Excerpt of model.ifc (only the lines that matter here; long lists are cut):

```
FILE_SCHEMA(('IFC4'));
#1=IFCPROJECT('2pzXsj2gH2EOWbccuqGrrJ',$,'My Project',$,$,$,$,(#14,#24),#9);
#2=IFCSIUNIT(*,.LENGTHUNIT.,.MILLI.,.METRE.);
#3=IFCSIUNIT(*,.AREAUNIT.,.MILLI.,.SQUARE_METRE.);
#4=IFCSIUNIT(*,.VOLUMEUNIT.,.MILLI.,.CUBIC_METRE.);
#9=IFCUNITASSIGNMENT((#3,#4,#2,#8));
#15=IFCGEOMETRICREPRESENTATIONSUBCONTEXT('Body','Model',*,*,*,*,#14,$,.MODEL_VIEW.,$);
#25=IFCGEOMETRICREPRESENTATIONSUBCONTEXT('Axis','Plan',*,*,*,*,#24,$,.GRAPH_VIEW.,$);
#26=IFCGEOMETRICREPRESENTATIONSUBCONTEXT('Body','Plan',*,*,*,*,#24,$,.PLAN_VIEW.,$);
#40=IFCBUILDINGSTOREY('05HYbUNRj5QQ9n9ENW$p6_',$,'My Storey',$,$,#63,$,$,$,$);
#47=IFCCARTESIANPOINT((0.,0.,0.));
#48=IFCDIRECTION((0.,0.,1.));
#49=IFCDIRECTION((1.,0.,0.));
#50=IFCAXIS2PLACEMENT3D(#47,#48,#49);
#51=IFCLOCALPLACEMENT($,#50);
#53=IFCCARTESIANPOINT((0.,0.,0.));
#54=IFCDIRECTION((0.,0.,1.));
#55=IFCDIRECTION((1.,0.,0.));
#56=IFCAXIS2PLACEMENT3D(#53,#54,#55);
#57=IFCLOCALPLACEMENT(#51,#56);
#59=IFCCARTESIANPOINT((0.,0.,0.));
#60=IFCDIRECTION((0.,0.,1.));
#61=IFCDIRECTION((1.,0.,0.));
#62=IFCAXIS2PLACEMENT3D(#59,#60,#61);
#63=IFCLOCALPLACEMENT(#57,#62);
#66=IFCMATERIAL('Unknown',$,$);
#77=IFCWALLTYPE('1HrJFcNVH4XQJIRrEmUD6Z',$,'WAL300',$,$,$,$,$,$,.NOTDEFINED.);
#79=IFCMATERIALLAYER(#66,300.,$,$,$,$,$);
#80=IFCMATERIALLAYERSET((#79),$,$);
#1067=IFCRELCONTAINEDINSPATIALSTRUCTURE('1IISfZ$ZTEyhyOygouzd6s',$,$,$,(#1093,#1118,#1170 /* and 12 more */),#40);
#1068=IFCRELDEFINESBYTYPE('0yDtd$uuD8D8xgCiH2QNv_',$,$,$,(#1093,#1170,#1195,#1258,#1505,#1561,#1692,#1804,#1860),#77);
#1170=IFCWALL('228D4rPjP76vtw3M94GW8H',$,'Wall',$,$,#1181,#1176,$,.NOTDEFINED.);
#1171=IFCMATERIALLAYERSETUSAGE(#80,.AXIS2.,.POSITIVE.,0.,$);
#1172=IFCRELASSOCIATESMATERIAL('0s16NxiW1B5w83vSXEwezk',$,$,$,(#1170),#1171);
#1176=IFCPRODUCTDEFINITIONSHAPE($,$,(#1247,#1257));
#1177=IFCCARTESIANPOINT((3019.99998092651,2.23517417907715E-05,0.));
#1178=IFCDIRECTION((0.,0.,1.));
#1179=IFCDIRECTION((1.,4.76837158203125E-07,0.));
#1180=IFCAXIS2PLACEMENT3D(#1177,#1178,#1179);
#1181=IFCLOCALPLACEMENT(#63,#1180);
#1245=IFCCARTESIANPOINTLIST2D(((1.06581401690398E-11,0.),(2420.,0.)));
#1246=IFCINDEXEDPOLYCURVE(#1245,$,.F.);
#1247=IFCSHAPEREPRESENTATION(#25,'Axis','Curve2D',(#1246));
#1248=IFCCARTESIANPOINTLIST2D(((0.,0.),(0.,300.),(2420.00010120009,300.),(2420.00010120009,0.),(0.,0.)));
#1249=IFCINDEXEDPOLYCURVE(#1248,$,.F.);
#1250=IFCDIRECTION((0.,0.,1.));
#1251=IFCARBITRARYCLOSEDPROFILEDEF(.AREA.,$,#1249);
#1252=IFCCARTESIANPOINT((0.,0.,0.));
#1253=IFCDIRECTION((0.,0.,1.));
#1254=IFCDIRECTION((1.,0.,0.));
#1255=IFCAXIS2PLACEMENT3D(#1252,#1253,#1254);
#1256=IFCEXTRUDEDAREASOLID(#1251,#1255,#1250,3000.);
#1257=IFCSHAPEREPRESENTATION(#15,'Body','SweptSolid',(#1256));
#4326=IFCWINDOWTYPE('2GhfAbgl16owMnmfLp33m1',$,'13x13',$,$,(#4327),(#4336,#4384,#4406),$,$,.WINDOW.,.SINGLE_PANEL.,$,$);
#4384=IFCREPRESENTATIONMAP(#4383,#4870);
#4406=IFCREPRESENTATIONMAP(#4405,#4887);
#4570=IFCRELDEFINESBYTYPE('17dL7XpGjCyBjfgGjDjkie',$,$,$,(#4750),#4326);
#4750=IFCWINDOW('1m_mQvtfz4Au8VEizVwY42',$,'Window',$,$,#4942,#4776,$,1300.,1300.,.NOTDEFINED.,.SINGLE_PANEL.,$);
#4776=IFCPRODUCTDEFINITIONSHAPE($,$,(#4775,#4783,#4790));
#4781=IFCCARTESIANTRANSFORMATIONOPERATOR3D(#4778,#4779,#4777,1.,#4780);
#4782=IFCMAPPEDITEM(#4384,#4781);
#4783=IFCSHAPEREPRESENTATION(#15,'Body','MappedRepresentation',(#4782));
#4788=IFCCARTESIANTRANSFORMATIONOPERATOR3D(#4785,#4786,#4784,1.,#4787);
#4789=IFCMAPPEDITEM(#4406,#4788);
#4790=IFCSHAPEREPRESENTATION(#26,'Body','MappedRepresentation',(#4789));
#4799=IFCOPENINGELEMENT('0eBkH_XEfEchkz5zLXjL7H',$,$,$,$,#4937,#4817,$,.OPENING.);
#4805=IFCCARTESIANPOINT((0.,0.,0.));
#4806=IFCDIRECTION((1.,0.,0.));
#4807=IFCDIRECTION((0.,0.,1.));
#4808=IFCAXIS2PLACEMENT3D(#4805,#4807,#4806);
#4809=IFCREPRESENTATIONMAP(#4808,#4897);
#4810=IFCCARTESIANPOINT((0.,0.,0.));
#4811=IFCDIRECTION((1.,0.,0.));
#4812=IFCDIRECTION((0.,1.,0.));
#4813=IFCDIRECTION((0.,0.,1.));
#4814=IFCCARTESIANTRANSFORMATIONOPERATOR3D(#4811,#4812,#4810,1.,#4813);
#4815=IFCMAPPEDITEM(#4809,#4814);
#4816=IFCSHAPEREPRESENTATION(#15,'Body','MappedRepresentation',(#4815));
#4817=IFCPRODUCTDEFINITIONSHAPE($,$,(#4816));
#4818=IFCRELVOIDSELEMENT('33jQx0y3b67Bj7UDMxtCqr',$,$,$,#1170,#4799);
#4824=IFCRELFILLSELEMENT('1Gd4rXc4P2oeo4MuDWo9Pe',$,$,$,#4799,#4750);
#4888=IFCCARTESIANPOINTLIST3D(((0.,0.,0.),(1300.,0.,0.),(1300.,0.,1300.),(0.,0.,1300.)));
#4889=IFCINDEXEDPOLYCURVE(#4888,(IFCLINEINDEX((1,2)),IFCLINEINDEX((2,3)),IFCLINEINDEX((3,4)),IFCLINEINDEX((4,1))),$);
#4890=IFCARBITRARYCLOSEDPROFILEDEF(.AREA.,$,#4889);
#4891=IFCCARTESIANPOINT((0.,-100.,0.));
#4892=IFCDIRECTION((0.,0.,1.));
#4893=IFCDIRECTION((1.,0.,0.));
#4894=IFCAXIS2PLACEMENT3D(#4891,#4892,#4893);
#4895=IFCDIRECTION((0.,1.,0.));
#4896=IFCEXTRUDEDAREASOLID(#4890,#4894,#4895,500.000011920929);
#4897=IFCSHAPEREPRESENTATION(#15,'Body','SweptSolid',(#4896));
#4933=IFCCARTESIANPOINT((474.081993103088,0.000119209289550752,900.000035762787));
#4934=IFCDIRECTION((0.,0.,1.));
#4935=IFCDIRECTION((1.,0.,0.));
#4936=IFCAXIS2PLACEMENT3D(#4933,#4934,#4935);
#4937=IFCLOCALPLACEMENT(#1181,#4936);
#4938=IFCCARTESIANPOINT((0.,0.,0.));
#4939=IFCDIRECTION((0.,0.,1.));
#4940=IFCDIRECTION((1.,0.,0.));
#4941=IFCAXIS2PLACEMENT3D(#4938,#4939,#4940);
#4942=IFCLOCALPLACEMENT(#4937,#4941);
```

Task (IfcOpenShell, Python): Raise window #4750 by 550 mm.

```python
import numpy as np
import ifcopenshell
import ifcopenshell.api.geometry
import ifcopenshell.util.placement
import ifcopenshell.util.unit

model = ifcopenshell.open("model.ifc")
unit_scale = ifcopenshell.util.unit.calculate_unit_scale(model)

window = model.by_guid("1m_mQvtfz4Au8VEizVwY42")
opening = window.FillsVoids[0].RelatingOpeningElement
dz = 0.55 / unit_scale

shift = np.array([0.0, 0.0, dz])
# The window is placed relative to its opening, so it follows when the opening moves.
matrix = ifcopenshell.util.placement.get_local_placement(opening.ObjectPlacement)
matrix[:3, 3] += shift
ifcopenshell.api.geometry.edit_object_placement(
    model, product=opening, matrix=matrix, is_si=False, should_transform_children=True
)

print(f"moved by {dz * unit_scale:+.3f} m")

model.write("model_rev.ifc")
```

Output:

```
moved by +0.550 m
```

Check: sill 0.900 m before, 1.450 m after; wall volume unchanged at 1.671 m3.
